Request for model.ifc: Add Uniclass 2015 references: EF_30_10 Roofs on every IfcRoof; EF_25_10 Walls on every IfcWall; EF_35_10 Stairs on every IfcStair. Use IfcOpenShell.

First a look at what the model holds.

```python
import ifcopenshell

model = ifcopenshell.open("model.ifc")
print(model.schema)
print("classifications:", [c.Name for c in model.by_type("IfcClassification")])
for ifc_class in ("IfcDoor", "IfcRoof", "IfcStair", "IfcWall", "IfcWindow"):
    print(ifc_class, len(model.by_type(ifc_class)))
```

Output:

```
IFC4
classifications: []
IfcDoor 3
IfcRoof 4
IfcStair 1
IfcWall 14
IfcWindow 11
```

```python
import ifcopenshell
import ifcopenshell.api.classification

model = ifcopenshell.open("model.ifc")

system = ifcopenshell.api.classification.add_classification(model, classification="Uniclass 2015")

codes = {
    "IfcRoof": ("EF_30_10", "Roofs"),
    "IfcWall": ("EF_25_10", "Walls"),
    "IfcStair": ("EF_35_10", "Stairs"),
}
for ifc_class, (code, name) in codes.items():
    products = model.by_type(ifc_class)
    ifcopenshell.api.classification.add_reference(
        model, products=products, classification=system, identification=code, name=name
    )
    print(code, len(products))

model.write("model_rev.ifc")
```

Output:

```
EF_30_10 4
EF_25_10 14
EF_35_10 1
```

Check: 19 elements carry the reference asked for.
